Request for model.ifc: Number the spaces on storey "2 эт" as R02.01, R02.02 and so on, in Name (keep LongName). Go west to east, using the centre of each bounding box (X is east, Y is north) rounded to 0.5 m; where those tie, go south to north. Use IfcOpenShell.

First a look at what the model holds.

```python
import ifcopenshell
import ifcopenshell.util.element
import ifcopenshell.util.placement

model = ifcopenshell.open("model.ifc")
print(model.schema)
storey = next(s for s in model.by_type("IfcBuildingStorey") if s.Name == "2 эт")
spaces = [e for e in ifcopenshell.util.element.get_decomposition(storey) if e.is_a("IfcSpace")]
for e in sorted(spaces, key=lambda e: e.id()):
    origin = ifcopenshell.util.placement.get_local_placement(e.ObjectPlacement)[:3, 3]
    print(e.id(), e.Name, e.LongName, origin.round(2) + 0.0, sep=" | ")
```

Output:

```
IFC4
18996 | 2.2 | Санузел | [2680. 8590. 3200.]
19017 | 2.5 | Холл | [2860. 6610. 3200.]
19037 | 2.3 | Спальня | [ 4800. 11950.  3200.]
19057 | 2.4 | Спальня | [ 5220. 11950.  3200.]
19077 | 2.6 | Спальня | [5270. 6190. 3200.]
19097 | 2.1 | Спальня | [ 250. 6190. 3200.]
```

```python
import ifcopenshell
import ifcopenshell.geom
import ifcopenshell.util.element
import ifcopenshell.util.shape

model = ifcopenshell.open("model.ifc")
settings = ifcopenshell.geom.settings()
settings.set("use-world-coords", True)


def centre(element):
    shape = ifcopenshell.geom.create_shape(settings, element)
    return ifcopenshell.util.shape.get_bbox_centroid(shape.geometry)


storey = next(s for s in model.by_type("IfcBuildingStorey") if s.Name == "2 эт")
spaces = [e for e in ifcopenshell.util.element.get_decomposition(storey) if e.is_a("IfcSpace")]

# Insertion points can sit at a corner or the storey origin, so sort by the geometry (in metres).
centres = {e: centre(e) for e in spaces}
spaces.sort(key=lambda e: (round(centres[e][0] / 0.5), centres[e][1]))

for i, e in enumerate(spaces, start=1):
    number = f"R02.{i:02d}"
    e.Name = number
    print(e.id(), number)

model.write("model-out.ifc")
```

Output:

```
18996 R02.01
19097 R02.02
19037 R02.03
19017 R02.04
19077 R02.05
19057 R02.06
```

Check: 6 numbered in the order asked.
